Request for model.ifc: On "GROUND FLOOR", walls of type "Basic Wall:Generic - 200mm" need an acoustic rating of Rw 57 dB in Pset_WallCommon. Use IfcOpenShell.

First a look at what the model holds.

```python
import ifcopenshell
import ifcopenshell.util.element

model = ifcopenshell.open("model.ifc")
print(model.schema)
storey = next(s for s in model.by_type("IfcBuildingStorey") if s.Name == "GROUND FLOOR")
walls = [e for e in ifcopenshell.util.element.get_decomposition(storey) if e.is_a("IfcWall")]
seen = {}
for e in walls:
    element_type = ifcopenshell.util.element.get_type(e)
    key = (element_type.Name if element_type != e and element_type else None, ifcopenshell.util.element.get_pset(e, "Pset_WallCommon", "AcousticRating"))
    seen[key] = seen.get(key, 0) + 1
for (name, value), count in sorted(seen.items(), key=str):
    print(count, "x", name, "|", value)
```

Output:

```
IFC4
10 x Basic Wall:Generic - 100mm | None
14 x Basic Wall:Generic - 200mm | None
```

```python
import ifcopenshell
import ifcopenshell.api.pset
import ifcopenshell.util.element

model = ifcopenshell.open("model.ifc")

storey = next(s for s in model.by_type("IfcBuildingStorey") if s.Name == "GROUND FLOOR")
walls = [e for e in ifcopenshell.util.element.get_decomposition(storey) if e.is_a("IfcWall")]

count = 0
for e in walls:
    element_type = ifcopenshell.util.element.get_type(e)
    if element_type in (None, e) or element_type.Name != "Basic Wall:Generic - 200mm":
        continue
    # add_pset returns the element's existing set when there is one.
    pset = ifcopenshell.api.pset.add_pset(model, product=e, name="Pset_WallCommon")
    ifcopenshell.api.pset.edit_pset(model, pset=pset, properties={"AcousticRating": "Rw 57 dB"})
    count += 1

print(count, "walls updated")

model.write("model_edited.ifc")
```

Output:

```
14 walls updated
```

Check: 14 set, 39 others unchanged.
